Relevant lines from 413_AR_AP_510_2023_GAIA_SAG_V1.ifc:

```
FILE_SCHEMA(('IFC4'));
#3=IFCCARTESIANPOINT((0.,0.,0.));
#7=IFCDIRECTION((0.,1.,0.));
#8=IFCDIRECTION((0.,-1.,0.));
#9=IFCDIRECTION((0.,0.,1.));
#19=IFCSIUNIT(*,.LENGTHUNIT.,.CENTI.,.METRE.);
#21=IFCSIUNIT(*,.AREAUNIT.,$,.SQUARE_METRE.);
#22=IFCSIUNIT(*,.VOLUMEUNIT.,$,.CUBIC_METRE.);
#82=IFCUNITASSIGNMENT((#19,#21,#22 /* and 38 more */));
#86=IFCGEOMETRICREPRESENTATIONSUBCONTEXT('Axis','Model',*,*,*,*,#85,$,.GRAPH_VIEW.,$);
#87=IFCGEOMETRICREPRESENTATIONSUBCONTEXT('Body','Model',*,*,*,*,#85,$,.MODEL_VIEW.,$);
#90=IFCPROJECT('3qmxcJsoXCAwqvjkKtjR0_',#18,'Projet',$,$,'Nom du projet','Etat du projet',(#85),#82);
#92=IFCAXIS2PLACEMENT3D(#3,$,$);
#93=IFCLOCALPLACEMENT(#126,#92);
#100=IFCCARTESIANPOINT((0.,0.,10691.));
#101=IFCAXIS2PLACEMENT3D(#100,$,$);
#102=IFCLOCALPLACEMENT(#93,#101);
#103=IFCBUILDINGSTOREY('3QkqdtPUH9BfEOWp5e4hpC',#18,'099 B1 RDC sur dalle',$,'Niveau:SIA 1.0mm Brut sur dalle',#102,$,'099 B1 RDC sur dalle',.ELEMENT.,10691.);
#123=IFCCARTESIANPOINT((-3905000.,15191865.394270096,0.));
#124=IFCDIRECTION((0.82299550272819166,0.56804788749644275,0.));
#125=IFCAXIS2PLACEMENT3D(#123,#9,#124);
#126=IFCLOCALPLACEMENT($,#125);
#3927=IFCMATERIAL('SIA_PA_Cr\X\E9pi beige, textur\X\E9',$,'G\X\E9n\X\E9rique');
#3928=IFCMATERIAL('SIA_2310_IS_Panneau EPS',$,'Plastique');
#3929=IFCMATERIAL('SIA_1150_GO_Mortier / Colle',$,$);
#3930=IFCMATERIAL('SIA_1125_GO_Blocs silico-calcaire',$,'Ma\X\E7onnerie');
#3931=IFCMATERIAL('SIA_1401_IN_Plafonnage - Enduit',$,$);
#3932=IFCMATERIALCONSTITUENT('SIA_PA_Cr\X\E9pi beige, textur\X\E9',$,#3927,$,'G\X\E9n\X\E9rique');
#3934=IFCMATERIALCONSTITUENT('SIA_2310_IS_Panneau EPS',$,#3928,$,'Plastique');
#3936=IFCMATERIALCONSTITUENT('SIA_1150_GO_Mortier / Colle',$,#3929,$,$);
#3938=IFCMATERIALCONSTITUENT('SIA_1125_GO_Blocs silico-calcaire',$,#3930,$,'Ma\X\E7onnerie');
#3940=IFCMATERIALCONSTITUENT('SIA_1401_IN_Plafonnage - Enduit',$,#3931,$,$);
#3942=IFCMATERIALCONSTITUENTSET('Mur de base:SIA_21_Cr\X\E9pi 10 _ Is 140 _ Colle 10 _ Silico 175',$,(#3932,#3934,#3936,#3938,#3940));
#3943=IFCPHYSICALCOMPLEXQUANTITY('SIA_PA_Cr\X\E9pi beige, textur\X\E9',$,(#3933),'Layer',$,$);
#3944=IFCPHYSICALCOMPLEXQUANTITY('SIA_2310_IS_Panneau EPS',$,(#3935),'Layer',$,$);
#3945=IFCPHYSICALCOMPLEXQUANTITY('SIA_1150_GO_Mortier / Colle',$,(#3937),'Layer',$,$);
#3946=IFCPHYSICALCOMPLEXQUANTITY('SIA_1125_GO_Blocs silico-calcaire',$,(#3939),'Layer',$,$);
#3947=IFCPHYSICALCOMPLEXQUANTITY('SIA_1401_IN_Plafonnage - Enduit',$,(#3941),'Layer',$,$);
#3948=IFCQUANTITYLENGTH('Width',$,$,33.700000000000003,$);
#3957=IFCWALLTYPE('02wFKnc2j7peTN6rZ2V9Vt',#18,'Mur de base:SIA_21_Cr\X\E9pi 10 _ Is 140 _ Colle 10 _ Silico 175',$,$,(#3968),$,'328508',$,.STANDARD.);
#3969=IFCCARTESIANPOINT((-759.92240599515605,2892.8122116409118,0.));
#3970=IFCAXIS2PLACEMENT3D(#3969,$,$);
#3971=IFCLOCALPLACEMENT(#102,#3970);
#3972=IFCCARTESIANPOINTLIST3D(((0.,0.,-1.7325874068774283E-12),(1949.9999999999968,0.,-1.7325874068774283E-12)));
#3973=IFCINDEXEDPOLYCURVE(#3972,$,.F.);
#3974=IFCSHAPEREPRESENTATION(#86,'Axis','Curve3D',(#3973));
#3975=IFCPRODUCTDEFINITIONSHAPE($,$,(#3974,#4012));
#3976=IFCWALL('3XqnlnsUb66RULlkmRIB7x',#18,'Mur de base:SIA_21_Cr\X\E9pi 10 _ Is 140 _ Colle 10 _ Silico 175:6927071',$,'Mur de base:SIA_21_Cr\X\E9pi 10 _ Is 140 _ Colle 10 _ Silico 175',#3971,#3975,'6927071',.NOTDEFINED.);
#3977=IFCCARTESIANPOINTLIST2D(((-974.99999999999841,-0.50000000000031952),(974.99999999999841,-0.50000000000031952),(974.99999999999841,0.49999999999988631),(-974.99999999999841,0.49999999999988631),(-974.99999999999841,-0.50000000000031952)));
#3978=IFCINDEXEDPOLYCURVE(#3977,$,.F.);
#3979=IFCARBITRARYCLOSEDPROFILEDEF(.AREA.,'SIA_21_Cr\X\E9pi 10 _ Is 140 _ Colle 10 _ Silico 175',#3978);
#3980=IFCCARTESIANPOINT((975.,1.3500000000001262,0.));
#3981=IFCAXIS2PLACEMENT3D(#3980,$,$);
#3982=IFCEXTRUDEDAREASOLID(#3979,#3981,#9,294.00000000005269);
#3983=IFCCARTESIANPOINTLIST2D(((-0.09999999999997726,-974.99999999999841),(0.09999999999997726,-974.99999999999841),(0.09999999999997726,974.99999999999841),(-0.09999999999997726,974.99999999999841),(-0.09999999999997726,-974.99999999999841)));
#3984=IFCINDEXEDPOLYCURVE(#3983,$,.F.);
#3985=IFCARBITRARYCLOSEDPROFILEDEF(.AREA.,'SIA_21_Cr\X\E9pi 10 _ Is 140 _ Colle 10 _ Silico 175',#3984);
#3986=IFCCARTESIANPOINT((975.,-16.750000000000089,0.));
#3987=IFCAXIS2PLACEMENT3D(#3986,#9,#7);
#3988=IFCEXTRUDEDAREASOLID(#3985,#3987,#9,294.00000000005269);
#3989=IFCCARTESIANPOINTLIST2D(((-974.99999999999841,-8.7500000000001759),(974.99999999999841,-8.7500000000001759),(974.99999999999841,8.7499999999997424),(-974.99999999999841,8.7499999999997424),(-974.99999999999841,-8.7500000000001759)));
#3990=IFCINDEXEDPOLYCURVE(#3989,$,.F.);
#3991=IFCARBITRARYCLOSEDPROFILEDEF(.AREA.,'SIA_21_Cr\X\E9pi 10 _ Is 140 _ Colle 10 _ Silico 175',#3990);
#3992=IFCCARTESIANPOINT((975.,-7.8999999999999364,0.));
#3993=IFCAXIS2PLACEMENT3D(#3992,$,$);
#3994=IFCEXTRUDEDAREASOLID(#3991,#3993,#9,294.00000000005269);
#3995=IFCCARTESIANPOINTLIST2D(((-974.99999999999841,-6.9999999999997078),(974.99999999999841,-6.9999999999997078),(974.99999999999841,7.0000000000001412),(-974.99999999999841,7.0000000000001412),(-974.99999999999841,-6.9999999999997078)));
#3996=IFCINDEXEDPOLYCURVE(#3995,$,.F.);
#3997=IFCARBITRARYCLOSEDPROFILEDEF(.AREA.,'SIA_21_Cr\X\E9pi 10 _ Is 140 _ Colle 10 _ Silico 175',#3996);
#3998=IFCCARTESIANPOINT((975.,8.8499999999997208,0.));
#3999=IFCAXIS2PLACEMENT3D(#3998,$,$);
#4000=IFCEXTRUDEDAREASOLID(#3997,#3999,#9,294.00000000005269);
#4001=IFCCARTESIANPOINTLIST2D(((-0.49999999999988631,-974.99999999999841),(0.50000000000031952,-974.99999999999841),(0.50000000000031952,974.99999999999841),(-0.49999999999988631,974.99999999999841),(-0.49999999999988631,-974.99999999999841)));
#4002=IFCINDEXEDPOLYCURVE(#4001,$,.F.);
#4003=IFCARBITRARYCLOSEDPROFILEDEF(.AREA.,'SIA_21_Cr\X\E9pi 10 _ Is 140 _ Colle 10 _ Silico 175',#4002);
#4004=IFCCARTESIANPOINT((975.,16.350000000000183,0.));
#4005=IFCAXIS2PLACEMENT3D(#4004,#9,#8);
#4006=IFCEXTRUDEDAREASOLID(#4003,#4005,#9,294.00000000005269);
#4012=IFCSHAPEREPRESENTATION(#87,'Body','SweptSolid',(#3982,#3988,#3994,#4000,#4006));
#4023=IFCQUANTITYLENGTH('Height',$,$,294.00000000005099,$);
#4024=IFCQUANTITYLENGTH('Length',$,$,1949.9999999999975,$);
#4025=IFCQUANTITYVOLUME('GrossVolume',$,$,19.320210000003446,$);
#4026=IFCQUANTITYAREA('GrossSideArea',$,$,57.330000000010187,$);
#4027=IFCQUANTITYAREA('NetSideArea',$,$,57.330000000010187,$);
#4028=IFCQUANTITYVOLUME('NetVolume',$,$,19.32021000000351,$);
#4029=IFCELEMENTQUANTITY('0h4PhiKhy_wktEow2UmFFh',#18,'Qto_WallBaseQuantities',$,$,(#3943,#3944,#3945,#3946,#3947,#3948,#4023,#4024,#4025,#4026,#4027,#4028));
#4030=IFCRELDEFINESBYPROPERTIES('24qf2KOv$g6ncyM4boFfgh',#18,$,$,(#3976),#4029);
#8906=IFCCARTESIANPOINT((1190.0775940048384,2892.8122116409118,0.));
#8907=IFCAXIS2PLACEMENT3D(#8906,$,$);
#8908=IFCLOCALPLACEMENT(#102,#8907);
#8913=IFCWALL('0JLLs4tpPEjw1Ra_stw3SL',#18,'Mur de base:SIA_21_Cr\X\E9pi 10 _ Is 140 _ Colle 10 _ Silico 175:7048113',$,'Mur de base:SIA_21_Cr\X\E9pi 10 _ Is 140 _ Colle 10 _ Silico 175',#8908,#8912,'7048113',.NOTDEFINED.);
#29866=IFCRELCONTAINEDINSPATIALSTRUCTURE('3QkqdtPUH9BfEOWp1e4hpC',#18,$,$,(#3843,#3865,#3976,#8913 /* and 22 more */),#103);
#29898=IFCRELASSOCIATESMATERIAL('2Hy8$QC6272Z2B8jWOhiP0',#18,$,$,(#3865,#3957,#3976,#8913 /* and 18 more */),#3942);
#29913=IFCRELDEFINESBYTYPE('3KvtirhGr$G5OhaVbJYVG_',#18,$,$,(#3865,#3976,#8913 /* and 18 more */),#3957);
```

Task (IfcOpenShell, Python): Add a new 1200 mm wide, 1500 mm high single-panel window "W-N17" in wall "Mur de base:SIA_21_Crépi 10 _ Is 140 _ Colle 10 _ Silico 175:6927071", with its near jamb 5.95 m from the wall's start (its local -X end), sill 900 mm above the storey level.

```python
import numpy as np
import ifcopenshell
import ifcopenshell.api.feature
import ifcopenshell.api.geometry
import ifcopenshell.api.pset
import ifcopenshell.api.root
import ifcopenshell.api.spatial
import ifcopenshell.geom
import ifcopenshell.util.element
import ifcopenshell.util.placement
import ifcopenshell.util.representation
import ifcopenshell.util.shape
import ifcopenshell.util.unit

model = ifcopenshell.open("413_AR_AP_510_2023_GAIA_SAG_V1.ifc")
unit_scale = ifcopenshell.util.unit.calculate_unit_scale(model)
area_scale = ifcopenshell.util.unit.calculate_unit_scale(model, "AREAUNIT")
volume_scale = ifcopenshell.util.unit.calculate_unit_scale(model, "VOLUMEUNIT")
settings = ifcopenshell.geom.settings()


def volume(element):
    """Net volume in cubic metres, openings subtracted."""
    shape = ifcopenshell.geom.create_shape(settings, element)
    return ifcopenshell.util.shape.get_volume(shape.geometry)


wall = model.by_guid("3XqnlnsUb66RULlkmRIB7x")
storey = ifcopenshell.util.element.get_container(wall, ifc_class="IfcBuildingStorey")
context = ifcopenshell.util.representation.get_context(model, "Model", "Body", "MODEL_VIEW")
before = volume(wall)

width, height, from_end, sill = 1.2, 1.5, 5.95, 0.9  # metres

# The wall runs along its own X axis, and the end named is its -X end.
wall_shape = ifcopenshell.geom.create_shape(settings, wall)
x, y, z = ifcopenshell.util.shape.get_vertices(wall_shape.geometry).T
start = x.min() + from_end
face, thickness = float(y.min()), float(y.max() - y.min())
wall_matrix = ifcopenshell.util.placement.get_local_placement(wall.ObjectPlacement)
level = ifcopenshell.util.placement.get_local_placement(storey.ObjectPlacement)[2, 3]


def in_wall(x, y):
    """Placement at x, y metres in the wall's axes, at sill height."""
    matrix = wall_matrix.copy()
    matrix[:, 3] = wall_matrix @ np.array([x / unit_scale, y / unit_scale, 0.0, 1.0])
    matrix[2, 3] = level + sill / unit_scale
    return matrix


# Opening: a box that overshoots both wall faces by 50 mm.
opening = ifcopenshell.api.root.create_entity(model, ifc_class="IfcOpeningElement", predefined_type="OPENING")
box = ifcopenshell.api.geometry.add_wall_representation(
    model, context=context, length=width, height=height, thickness=thickness + 0.1
)
ifcopenshell.api.geometry.assign_representation(model, product=opening, representation=box)
ifcopenshell.api.geometry.edit_object_placement(model, product=opening, matrix=in_wall(start, face - 0.05), is_si=False)
ifcopenshell.api.feature.add_feature(model, feature=opening, element=wall)

window = ifcopenshell.api.root.create_entity(model, ifc_class="IfcWindow", name="W-N17", predefined_type="WINDOW")
window.OverallWidth, window.OverallHeight = width / unit_scale, height / unit_scale
window.PartitioningType = "SINGLE_PANEL"
body = ifcopenshell.api.geometry.add_window_representation(
    model,
    context=context,
    overall_width=window.OverallWidth,
    overall_height=window.OverallHeight,
    partition_type="SINGLE_PANEL",
)
ifcopenshell.api.geometry.assign_representation(model, product=window, representation=body)
ifcopenshell.api.spatial.assign_container(model, products=[window], relating_structure=storey)
ifcopenshell.api.feature.add_filling(model, opening=opening, element=window)

# Centre the window in the wall's thickness.
ifcopenshell.api.geometry.edit_object_placement(model, product=window, matrix=in_wall(start, face), is_si=False)
window_shape = ifcopenshell.geom.create_shape(settings, window)
depth = ifcopenshell.util.shape.get_vertices(window_shape.geometry)[:, 1]
offset = face + thickness / 2 - (depth.min() + depth.max()) / 2
ifcopenshell.api.geometry.edit_object_placement(model, product=window, matrix=in_wall(start, offset), is_si=False)

after = volume(wall)

# Update the wall's stored quantities.
qto = model.by_id(ifcopenshell.util.element.get_pset(wall, "Qto_WallBaseQuantities", should_inherit=False)["id"])
ifcopenshell.api.pset.edit_qto(model, qto=qto, properties={
    "NetSideArea": after / thickness / area_scale,
    "NetVolume": after / volume_scale,
})

print(f"wall volume {before:.3f} -> {after:.3f} m3")

model.write("413_AR_AP_510_2023_GAIA_SAG_V1_rev.ifc")
```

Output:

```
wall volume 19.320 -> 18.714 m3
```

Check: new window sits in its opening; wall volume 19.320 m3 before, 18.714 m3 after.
